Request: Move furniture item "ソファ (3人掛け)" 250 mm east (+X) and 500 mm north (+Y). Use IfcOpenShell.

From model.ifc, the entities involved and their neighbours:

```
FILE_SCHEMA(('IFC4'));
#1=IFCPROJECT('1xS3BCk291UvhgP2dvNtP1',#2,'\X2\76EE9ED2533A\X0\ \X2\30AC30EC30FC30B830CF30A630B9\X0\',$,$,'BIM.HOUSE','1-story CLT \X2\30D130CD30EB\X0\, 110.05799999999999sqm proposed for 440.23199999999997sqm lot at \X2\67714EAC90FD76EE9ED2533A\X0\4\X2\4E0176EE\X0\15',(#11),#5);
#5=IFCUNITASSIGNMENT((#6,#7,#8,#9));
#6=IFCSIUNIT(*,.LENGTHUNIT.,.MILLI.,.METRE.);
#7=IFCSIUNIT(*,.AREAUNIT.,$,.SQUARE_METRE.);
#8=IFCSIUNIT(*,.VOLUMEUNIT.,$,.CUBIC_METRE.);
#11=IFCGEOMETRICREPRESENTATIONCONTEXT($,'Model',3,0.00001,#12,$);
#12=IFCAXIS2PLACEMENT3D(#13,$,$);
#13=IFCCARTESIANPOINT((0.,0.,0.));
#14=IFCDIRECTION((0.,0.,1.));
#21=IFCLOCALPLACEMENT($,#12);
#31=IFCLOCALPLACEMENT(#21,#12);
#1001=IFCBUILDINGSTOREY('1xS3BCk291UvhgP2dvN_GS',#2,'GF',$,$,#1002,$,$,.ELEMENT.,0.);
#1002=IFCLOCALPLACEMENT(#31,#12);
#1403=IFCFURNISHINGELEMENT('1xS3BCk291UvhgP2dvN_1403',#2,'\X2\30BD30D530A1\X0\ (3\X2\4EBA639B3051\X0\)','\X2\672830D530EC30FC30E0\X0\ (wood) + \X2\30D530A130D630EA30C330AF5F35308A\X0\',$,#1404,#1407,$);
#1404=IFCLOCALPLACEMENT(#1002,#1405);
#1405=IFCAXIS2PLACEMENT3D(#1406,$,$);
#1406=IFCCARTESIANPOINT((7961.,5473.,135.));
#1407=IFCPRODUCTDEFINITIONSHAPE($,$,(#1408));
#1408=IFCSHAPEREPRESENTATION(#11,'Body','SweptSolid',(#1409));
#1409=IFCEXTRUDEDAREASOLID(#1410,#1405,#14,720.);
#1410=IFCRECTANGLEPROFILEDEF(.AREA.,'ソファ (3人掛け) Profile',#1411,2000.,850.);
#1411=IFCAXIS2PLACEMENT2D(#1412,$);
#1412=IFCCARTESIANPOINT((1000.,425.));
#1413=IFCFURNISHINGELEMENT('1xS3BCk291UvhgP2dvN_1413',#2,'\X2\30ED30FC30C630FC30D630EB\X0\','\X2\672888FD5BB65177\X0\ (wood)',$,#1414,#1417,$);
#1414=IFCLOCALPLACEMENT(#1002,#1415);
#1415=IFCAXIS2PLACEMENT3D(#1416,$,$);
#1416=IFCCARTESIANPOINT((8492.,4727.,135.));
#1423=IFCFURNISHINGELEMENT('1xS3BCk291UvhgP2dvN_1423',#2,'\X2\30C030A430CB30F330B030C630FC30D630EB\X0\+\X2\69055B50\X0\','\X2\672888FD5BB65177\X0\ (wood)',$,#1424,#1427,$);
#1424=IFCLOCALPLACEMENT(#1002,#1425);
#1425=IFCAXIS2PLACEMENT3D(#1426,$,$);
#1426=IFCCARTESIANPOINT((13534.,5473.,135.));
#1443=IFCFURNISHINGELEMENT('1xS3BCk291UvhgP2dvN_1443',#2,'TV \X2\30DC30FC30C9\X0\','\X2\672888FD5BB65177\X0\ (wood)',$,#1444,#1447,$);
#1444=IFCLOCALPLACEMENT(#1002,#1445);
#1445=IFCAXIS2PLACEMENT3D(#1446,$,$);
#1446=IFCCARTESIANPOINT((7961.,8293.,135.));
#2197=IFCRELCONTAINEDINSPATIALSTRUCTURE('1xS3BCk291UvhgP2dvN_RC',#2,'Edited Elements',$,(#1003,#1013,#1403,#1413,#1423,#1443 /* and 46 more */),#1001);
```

```python
import ifcopenshell
import ifcopenshell.api.geometry
import ifcopenshell.util.placement

model = ifcopenshell.open("model.ifc")

item = model.by_guid("1xS3BCk291UvhgP2dvN_1403")
matrix = ifcopenshell.util.placement.get_local_placement(item.ObjectPlacement)
matrix[0, 3] += 250.0
matrix[1, 3] += 500.0
ifcopenshell.api.geometry.edit_object_placement(model, product=item, matrix=matrix, is_si=False)

print(ifcopenshell.util.placement.get_local_placement(item.ObjectPlacement).round(3) + 0.0)

model.write("model_v2.ifc")
```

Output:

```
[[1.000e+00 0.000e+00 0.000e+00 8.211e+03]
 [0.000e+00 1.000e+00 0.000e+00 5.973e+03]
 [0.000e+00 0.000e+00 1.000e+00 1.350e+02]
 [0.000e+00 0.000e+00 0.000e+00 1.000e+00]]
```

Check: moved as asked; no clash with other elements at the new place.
